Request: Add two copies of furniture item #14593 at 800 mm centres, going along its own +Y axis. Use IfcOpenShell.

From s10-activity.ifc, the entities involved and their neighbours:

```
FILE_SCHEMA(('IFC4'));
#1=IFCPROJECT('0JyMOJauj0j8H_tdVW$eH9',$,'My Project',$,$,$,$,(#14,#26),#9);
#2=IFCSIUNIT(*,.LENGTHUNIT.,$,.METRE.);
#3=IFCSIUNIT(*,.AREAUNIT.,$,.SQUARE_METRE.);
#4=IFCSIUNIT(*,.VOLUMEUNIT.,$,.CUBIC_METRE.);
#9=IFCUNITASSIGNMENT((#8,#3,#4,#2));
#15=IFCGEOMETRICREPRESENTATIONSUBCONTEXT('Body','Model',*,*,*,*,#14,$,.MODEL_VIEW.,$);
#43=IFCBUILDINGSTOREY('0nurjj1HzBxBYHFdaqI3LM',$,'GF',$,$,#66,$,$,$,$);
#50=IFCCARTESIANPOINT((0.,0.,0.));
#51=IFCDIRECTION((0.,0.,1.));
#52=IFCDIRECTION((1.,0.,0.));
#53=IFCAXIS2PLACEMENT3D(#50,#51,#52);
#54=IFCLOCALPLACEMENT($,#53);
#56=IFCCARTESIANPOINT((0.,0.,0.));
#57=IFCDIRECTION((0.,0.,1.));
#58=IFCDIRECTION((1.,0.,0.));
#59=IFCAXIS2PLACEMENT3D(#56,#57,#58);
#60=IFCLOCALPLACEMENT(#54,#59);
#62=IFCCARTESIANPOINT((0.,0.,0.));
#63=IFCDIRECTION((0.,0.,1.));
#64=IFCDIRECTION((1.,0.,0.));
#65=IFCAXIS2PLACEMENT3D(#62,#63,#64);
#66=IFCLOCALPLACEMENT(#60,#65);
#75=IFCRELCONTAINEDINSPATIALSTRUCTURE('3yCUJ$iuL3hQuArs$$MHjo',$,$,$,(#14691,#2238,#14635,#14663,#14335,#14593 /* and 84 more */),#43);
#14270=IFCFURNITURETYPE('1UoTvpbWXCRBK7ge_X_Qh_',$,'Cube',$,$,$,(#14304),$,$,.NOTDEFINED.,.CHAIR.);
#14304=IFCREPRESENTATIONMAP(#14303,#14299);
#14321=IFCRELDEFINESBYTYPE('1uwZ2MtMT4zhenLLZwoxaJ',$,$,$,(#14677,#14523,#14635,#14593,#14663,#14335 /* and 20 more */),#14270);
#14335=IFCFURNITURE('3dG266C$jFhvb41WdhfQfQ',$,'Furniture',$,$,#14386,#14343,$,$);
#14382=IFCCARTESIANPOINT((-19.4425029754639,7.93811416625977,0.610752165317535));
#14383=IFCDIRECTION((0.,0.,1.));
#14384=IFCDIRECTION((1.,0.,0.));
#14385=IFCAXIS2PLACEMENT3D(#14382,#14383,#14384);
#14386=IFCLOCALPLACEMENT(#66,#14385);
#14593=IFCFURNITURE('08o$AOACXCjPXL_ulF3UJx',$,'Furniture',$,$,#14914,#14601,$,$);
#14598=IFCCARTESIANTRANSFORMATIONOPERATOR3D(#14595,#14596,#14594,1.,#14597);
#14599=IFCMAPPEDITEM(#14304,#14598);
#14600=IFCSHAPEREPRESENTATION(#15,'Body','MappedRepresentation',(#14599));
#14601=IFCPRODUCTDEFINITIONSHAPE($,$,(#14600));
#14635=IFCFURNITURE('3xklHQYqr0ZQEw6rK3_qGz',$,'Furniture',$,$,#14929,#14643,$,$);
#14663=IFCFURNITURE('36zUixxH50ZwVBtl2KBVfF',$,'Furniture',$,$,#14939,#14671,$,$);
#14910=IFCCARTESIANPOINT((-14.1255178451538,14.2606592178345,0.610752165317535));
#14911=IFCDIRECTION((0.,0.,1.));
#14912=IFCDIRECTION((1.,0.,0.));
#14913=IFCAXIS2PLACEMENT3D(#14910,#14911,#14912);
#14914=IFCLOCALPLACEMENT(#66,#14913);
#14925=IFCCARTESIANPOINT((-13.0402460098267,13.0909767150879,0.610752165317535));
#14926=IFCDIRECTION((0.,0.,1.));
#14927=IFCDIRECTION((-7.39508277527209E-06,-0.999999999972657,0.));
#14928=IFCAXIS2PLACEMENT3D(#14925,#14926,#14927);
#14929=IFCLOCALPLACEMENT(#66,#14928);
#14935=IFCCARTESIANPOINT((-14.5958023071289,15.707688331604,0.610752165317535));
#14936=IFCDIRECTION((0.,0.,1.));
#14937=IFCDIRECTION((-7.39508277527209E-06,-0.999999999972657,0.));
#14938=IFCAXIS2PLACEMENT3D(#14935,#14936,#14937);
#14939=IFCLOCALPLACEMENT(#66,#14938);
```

```python
import ifcopenshell
import ifcopenshell.api.geometry
import ifcopenshell.api.root
import ifcopenshell.util.element
import ifcopenshell.util.placement
import ifcopenshell.util.unit

model = ifcopenshell.open("s10-activity.ifc")
unit_scale = ifcopenshell.util.unit.calculate_unit_scale(model)

source = model.by_guid("08o$AOACXCjPXL_ulF3UJx")
base = ifcopenshell.util.placement.get_local_placement(source.ObjectPlacement)
step = base[:3, 1] * 0.8 / unit_scale

for i in range(1, 3):
    copy = ifcopenshell.api.root.copy_class(model, product=source)
    copy.Representation = ifcopenshell.util.element.copy_deep(
        model, source.Representation, exclude=["IfcGeometricRepresentationContext", "IfcRepresentationMap"]
    )
    matrix = base.copy()
    matrix[:3, 3] += i * step
    print("added at", matrix[:3, 3].round(3) + 0.0)
    ifcopenshell.api.geometry.edit_object_placement(model, product=copy, matrix=matrix, is_si=False)

model.write("s10-activity_edited.ifc")
```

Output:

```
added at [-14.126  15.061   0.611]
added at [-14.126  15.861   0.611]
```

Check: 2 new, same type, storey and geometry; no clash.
